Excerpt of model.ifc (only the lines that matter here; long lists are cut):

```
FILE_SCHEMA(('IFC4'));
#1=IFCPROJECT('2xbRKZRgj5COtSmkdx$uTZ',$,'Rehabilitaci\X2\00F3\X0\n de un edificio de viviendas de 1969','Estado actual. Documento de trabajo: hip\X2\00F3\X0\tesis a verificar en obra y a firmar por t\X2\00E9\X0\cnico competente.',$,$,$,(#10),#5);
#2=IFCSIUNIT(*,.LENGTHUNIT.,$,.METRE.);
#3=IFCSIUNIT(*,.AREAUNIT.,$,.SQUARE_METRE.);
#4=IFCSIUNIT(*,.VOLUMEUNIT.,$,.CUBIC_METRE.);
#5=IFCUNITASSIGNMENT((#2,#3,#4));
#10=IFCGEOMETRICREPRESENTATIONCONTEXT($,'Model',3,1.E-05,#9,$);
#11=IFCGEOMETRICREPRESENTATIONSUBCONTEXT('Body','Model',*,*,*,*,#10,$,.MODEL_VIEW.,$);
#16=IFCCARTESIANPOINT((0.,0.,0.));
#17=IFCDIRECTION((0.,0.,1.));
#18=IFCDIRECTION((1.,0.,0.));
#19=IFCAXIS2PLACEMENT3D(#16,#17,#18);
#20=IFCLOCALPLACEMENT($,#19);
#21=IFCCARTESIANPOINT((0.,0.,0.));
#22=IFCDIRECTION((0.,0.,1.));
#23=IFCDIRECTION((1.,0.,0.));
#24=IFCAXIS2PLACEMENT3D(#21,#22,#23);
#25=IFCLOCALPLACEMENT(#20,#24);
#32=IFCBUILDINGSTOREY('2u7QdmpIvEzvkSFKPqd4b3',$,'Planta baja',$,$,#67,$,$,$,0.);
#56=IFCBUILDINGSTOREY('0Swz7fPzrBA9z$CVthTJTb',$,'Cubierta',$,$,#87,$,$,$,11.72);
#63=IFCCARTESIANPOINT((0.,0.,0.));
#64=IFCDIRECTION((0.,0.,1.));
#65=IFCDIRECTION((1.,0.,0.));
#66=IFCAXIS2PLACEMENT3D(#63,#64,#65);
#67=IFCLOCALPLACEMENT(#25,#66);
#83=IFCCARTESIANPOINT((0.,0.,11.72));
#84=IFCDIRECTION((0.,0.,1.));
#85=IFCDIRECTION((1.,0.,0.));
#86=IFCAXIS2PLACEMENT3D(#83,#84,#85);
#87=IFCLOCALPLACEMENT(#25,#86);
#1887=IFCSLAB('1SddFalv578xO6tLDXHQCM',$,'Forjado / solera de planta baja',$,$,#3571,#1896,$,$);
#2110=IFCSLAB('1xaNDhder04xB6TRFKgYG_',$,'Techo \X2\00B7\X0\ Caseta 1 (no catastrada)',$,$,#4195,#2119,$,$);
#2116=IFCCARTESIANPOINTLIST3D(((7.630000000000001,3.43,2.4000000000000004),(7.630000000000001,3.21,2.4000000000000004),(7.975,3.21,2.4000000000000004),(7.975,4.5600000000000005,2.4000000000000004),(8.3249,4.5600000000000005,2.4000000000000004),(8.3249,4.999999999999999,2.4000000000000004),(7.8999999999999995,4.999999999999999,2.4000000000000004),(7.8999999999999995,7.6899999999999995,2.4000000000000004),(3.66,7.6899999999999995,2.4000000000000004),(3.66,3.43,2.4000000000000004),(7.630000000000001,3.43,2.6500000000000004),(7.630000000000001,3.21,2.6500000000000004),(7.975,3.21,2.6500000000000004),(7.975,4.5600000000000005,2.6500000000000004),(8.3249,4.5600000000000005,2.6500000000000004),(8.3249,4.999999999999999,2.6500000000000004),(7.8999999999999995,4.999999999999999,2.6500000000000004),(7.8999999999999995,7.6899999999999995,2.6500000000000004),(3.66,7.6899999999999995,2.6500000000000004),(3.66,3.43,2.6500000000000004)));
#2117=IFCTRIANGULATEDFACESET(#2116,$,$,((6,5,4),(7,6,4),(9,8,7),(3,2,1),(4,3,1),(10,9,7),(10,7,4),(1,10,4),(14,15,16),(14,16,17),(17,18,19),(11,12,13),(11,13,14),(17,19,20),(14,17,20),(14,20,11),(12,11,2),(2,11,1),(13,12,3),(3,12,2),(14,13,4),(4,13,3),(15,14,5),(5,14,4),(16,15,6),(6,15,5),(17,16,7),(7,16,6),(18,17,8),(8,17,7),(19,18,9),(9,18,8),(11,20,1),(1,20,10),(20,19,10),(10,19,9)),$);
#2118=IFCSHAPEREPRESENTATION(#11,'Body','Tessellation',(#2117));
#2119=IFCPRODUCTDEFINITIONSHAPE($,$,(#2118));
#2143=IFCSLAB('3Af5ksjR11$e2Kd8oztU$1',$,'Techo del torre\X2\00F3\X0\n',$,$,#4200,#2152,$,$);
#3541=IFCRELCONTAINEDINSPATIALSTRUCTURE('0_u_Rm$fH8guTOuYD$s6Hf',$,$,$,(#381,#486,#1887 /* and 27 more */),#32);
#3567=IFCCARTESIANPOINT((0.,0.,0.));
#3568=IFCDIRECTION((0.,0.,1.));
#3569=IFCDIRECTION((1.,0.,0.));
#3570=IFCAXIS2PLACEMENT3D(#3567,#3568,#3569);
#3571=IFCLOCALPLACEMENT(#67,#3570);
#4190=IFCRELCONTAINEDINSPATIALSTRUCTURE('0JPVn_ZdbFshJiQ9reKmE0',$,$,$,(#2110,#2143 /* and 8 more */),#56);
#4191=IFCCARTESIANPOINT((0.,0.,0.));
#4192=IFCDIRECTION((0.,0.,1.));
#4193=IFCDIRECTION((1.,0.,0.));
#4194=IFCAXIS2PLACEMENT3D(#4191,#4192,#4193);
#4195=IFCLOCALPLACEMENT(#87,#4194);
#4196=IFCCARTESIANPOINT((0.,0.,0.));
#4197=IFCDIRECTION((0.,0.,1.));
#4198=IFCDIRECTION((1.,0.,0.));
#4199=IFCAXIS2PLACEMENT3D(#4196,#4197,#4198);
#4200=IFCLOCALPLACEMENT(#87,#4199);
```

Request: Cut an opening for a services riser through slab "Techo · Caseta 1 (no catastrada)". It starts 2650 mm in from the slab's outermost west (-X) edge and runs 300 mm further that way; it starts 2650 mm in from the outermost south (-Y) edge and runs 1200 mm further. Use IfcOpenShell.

```python
import numpy as np
import ifcopenshell
import ifcopenshell.api.feature
import ifcopenshell.api.geometry
import ifcopenshell.api.root
import ifcopenshell.geom
import ifcopenshell.util.placement
import ifcopenshell.util.representation
import ifcopenshell.util.shape
import ifcopenshell.util.unit

model = ifcopenshell.open("model.ifc")
unit_scale = ifcopenshell.util.unit.calculate_unit_scale(model)
settings = ifcopenshell.geom.settings()


def volume(element):
    """Net volume in cubic metres, openings subtracted."""
    shape = ifcopenshell.geom.create_shape(settings, element)
    return ifcopenshell.util.shape.get_volume(shape.geometry)


slab = model.by_guid("1xaNDhder04xB6TRFKgYG_")
before = volume(slab)

# Extent in the slab's own axes, in metres. The edges named are its -X and -Y sides.
slab_shape = ifcopenshell.geom.create_shape(settings, slab)
vertices = ifcopenshell.util.shape.get_vertices(slab_shape.geometry)
x_min, y_min, bottom = vertices.min(axis=0)
top = vertices[:, 2].max()

opening = ifcopenshell.api.root.create_entity(model, ifc_class="IfcOpeningElement", name="Services riser opening", predefined_type="OPENING")
context = ifcopenshell.util.representation.get_context(model, "Model", "Body", "MODEL_VIEW")
width, depth = 0.3, 1.2
outline = [(0.0, 0.0), (width, 0.0), (width, depth), (0.0, depth), (0.0, 0.0)]
# Overshoot both faces by 50 mm so the cut is clean.
shape = ifcopenshell.api.geometry.add_slab_representation(
    model, context=context, depth=top - bottom + 0.1, polyline=outline
)
ifcopenshell.api.geometry.assign_representation(model, product=opening, representation=shape)

matrix = ifcopenshell.util.placement.get_local_placement(slab.ObjectPlacement)
matrix[:, 3] = matrix @ np.append(np.array([x_min + 2.65, y_min + 2.65, bottom - 0.05]) / unit_scale, 1.0)
ifcopenshell.api.geometry.edit_object_placement(model, product=opening, matrix=matrix, is_si=False)
ifcopenshell.api.feature.add_feature(model, feature=opening, element=slab)

after = volume(slab)

print(f"slab volume {before:.3f} -> {after:.3f} m3")

model.write("model-out.ifc")
```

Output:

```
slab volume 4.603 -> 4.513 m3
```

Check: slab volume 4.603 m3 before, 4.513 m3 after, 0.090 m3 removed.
